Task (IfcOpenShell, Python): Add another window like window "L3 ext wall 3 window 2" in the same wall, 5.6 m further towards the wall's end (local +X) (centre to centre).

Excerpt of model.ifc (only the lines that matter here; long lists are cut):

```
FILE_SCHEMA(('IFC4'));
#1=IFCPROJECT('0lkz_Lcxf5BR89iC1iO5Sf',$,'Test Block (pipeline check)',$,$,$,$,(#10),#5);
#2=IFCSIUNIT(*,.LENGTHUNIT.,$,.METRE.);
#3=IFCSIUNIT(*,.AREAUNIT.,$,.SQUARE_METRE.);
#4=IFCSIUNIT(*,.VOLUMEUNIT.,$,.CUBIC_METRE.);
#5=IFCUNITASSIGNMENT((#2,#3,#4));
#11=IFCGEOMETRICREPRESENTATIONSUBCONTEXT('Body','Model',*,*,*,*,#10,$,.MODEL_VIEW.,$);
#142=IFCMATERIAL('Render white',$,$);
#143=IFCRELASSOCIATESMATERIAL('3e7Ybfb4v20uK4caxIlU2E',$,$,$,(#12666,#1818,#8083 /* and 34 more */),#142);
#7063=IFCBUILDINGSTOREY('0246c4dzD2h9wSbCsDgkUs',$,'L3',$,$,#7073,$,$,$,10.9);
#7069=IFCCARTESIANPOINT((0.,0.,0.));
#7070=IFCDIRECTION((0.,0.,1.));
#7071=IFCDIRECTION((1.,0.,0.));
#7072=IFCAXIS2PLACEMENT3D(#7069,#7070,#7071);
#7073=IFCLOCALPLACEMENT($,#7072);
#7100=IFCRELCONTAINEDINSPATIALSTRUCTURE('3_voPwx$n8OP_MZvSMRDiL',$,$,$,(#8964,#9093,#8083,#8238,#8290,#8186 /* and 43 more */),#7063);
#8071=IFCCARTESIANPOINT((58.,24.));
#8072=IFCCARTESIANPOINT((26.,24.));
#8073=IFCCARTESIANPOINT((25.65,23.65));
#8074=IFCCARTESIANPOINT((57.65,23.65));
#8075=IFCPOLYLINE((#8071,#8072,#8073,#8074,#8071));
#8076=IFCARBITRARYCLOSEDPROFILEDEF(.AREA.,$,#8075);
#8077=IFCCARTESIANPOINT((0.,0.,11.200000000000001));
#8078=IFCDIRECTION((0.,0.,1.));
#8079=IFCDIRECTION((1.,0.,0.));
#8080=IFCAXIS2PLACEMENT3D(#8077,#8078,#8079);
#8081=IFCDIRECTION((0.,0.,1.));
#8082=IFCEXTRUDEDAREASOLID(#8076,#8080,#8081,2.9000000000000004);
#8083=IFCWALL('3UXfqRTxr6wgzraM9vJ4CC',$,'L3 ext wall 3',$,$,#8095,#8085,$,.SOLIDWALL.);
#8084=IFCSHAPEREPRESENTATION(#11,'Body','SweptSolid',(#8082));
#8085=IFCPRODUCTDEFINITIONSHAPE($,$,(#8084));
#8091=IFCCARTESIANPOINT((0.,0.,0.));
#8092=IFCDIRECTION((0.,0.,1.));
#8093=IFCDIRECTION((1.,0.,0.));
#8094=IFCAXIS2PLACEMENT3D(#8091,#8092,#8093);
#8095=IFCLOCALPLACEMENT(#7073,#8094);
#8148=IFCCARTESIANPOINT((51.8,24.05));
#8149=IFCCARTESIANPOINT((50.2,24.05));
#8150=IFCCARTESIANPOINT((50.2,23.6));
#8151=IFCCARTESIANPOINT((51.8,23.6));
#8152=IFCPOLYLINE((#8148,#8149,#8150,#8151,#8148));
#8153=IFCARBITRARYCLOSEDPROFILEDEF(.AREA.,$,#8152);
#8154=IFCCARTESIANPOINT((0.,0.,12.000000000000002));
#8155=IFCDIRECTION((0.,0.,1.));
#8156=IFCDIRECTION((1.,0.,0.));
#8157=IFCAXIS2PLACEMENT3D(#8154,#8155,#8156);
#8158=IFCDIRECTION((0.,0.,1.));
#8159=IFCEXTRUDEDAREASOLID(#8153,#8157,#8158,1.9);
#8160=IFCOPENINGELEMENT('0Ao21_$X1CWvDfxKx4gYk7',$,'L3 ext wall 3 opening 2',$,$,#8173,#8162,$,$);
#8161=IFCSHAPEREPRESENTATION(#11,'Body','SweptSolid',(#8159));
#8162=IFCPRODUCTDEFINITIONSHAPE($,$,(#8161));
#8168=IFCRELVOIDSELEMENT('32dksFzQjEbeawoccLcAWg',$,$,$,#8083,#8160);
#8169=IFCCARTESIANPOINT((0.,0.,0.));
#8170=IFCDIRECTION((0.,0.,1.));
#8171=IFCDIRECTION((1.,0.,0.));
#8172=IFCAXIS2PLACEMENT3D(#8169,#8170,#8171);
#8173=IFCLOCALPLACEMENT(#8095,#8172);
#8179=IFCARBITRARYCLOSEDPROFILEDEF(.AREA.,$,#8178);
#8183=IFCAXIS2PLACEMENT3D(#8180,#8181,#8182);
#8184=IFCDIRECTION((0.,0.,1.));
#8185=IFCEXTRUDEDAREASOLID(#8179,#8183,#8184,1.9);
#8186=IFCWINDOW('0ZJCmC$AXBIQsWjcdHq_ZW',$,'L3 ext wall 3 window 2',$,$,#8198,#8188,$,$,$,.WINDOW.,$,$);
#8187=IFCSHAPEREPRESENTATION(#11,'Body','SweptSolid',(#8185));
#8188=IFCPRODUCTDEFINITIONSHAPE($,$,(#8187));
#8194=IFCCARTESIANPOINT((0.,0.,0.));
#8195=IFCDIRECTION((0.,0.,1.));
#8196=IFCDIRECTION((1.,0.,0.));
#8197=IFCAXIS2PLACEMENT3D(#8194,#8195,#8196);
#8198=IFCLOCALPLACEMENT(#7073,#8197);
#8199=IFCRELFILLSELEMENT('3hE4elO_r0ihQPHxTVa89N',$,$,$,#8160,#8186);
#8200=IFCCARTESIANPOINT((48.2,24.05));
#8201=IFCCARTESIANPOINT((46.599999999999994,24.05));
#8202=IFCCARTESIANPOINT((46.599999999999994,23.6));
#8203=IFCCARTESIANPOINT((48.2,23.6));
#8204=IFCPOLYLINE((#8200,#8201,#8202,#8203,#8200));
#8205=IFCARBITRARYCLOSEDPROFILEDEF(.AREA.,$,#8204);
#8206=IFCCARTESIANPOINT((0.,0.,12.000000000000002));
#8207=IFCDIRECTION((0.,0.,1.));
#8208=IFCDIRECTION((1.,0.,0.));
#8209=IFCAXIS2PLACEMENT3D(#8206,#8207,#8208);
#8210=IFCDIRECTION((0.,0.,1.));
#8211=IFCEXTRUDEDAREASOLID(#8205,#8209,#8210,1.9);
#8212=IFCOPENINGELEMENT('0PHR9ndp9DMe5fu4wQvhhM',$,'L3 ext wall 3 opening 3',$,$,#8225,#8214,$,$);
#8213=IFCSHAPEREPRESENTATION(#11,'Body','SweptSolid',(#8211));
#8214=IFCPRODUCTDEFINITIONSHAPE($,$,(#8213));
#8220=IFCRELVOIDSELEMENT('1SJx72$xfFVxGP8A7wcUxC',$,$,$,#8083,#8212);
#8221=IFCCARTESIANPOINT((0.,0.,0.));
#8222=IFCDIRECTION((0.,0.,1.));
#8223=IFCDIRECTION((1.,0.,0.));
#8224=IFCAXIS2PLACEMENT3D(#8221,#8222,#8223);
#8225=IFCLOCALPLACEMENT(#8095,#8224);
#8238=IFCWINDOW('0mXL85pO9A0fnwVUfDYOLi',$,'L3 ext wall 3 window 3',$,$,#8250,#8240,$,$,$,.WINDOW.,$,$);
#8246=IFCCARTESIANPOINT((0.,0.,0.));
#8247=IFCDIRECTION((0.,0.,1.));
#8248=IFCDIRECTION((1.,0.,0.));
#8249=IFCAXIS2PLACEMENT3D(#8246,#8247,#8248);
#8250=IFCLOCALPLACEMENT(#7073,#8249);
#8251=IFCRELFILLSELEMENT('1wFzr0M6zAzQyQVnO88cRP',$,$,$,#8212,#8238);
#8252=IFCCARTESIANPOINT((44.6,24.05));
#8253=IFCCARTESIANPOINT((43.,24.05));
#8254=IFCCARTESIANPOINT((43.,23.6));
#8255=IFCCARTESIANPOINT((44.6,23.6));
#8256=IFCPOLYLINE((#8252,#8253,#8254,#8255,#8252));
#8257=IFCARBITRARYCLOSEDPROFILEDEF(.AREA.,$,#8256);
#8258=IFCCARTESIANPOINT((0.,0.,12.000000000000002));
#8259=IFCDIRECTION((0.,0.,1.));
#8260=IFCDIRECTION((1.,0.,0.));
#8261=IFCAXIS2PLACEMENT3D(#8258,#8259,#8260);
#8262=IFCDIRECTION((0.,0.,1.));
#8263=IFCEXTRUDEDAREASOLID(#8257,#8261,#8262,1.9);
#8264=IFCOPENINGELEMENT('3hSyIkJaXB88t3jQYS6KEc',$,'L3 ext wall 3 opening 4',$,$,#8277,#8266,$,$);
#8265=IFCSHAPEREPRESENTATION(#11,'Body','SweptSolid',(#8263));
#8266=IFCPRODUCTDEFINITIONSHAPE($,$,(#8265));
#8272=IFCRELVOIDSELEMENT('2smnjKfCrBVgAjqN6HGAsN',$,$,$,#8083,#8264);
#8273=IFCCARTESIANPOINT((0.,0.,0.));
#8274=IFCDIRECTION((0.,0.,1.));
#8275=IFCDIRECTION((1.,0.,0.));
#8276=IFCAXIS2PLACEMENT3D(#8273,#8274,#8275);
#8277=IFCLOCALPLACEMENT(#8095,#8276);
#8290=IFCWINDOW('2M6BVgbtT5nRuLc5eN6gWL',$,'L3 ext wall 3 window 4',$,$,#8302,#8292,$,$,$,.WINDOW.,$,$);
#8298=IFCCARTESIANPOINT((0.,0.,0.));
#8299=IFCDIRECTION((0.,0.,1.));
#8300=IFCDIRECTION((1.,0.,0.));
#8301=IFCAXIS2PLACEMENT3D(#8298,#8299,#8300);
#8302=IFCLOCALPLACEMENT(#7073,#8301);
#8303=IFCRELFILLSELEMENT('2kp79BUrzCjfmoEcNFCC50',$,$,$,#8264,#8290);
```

```python
import ifcopenshell
import ifcopenshell.api.feature
import ifcopenshell.api.geometry
import ifcopenshell.api.root
import ifcopenshell.geom
import ifcopenshell.util.element
import ifcopenshell.util.placement
import ifcopenshell.util.shape

model = ifcopenshell.open("model.ifc")
settings = ifcopenshell.geom.settings()


def volume(element):
    """Net volume in cubic metres, openings subtracted."""
    shape = ifcopenshell.geom.create_shape(settings, element)
    return ifcopenshell.util.shape.get_volume(shape.geometry)


window = model.by_id(8186)
opening = window.FillsVoids[0].RelatingOpeningElement
wall = opening.VoidsElements[0].RelatingBuildingElement
before = volume(wall)
shift = ifcopenshell.util.placement.get_local_placement(wall.ObjectPlacement)[:3, 0] * 5.6

# copy_class copies the void relationship, type, container and properties, but no geometry.
new_opening = ifcopenshell.api.root.copy_class(model, product=opening)
new_opening.Representation = ifcopenshell.util.element.copy_deep(
    model, opening.Representation, exclude=["IfcGeometricRepresentationContext", "IfcRepresentationMap"]
)
new_window = ifcopenshell.api.root.copy_class(model, product=window)
new_window.Representation = ifcopenshell.util.element.copy_deep(
    model, window.Representation, exclude=["IfcGeometricRepresentationContext", "IfcRepresentationMap"]
)
ifcopenshell.api.feature.add_filling(model, opening=new_opening, element=new_window)

for old, new in ((opening, new_opening), (window, new_window)):
    matrix = ifcopenshell.util.placement.get_local_placement(old.ObjectPlacement)
    matrix[:3, 3] += shift
    ifcopenshell.api.geometry.edit_object_placement(model, product=new, matrix=matrix, is_si=False)

after = volume(wall)

print(f"wall volume {before:.3f} -> {after:.3f} m3")

model.write("model_rev.ifc")
```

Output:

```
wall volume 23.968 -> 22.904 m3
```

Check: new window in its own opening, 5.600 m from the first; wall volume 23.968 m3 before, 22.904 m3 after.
